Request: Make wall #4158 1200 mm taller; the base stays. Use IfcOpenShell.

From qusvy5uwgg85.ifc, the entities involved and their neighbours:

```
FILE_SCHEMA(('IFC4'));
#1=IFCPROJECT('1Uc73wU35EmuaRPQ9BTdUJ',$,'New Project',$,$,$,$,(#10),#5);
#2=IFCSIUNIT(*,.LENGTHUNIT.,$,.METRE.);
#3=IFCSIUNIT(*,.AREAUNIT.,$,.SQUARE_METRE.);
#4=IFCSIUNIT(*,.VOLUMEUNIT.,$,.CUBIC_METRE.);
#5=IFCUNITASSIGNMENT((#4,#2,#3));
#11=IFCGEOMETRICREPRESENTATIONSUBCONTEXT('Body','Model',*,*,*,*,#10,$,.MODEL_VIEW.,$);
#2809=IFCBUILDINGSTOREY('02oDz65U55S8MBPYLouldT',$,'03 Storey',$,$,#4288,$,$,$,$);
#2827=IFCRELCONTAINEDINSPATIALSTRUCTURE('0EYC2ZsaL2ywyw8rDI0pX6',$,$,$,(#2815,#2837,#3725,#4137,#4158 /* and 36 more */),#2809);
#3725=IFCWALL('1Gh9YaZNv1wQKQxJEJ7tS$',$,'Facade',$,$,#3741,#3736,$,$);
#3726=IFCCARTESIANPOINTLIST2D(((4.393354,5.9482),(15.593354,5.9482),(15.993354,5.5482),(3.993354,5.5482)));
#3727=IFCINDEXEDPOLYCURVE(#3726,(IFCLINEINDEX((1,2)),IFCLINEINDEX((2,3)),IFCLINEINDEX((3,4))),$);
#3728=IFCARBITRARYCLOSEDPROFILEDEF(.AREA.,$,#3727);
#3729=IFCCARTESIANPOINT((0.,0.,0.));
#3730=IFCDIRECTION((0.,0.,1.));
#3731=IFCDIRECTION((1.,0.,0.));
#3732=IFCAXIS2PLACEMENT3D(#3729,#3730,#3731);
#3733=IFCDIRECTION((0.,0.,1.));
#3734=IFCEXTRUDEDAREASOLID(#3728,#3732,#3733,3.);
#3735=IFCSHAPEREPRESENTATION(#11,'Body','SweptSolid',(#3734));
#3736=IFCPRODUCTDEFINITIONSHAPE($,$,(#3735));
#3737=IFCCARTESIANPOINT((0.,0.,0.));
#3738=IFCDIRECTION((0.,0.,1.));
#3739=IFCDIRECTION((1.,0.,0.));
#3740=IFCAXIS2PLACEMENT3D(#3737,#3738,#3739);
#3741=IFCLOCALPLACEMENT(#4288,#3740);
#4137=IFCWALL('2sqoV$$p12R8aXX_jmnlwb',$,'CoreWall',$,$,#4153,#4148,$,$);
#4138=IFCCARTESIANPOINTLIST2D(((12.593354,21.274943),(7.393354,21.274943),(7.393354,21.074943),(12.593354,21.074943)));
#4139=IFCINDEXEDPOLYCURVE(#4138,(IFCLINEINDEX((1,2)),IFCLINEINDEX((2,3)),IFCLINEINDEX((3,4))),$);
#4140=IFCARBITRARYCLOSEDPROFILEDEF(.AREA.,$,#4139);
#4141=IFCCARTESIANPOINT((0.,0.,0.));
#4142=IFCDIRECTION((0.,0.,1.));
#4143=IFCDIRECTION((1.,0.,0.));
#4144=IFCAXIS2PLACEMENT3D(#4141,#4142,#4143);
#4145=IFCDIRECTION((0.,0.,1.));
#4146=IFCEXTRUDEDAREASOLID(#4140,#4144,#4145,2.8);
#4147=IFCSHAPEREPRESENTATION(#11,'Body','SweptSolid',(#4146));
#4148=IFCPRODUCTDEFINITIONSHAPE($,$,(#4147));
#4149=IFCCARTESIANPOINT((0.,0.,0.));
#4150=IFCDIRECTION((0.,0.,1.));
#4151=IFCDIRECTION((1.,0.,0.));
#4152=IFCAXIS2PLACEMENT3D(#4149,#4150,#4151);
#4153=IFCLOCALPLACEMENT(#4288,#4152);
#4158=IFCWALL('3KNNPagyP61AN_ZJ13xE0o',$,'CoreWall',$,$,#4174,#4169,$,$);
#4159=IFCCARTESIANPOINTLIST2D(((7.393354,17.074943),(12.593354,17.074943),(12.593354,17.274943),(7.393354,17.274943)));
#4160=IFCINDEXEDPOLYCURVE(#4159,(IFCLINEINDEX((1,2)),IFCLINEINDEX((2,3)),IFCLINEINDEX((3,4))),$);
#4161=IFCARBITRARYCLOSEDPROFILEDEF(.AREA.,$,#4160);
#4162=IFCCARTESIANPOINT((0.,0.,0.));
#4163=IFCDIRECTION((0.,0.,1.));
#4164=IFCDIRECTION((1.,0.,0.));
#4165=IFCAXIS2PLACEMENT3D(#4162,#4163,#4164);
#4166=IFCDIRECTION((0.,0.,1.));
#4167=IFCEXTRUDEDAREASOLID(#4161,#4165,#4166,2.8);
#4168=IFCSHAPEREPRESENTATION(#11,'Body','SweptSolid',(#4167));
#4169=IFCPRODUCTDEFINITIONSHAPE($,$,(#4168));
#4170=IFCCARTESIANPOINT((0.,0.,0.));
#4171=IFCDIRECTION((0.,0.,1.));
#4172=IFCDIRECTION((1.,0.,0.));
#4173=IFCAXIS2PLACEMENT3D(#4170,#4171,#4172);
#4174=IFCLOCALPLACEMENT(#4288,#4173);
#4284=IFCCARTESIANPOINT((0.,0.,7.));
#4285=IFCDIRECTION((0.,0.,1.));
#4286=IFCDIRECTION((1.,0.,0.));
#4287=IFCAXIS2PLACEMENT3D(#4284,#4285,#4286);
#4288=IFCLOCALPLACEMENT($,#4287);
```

```python
import ifcopenshell
import ifcopenshell.geom
import ifcopenshell.util.representation
import ifcopenshell.util.shape
import ifcopenshell.util.unit

model = ifcopenshell.open("qusvy5uwgg85.ifc")
unit_scale = ifcopenshell.util.unit.calculate_unit_scale(model)
settings = ifcopenshell.geom.settings()


def volume(element):
    """Net volume in cubic metres, openings subtracted."""
    shape = ifcopenshell.geom.create_shape(settings, element)
    return ifcopenshell.util.shape.get_volume(shape.geometry)


wall = model.by_guid("3KNNPagyP61AN_ZJ13xE0o")
before = volume(wall)

body = ifcopenshell.util.representation.get_representation(wall, "Model", "Body")
solid = body.Items[0]
old_height = solid.Depth
solid.Depth += 1.2 / unit_scale
after = volume(wall)

print(f"height {old_height:g} -> {solid.Depth:g}, volume {before:.3f} -> {after:.3f} m3")

model.write("qusvy5uwgg85_rev.ifc")
```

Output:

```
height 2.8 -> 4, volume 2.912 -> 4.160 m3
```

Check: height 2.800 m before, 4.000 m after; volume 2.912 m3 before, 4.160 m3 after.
